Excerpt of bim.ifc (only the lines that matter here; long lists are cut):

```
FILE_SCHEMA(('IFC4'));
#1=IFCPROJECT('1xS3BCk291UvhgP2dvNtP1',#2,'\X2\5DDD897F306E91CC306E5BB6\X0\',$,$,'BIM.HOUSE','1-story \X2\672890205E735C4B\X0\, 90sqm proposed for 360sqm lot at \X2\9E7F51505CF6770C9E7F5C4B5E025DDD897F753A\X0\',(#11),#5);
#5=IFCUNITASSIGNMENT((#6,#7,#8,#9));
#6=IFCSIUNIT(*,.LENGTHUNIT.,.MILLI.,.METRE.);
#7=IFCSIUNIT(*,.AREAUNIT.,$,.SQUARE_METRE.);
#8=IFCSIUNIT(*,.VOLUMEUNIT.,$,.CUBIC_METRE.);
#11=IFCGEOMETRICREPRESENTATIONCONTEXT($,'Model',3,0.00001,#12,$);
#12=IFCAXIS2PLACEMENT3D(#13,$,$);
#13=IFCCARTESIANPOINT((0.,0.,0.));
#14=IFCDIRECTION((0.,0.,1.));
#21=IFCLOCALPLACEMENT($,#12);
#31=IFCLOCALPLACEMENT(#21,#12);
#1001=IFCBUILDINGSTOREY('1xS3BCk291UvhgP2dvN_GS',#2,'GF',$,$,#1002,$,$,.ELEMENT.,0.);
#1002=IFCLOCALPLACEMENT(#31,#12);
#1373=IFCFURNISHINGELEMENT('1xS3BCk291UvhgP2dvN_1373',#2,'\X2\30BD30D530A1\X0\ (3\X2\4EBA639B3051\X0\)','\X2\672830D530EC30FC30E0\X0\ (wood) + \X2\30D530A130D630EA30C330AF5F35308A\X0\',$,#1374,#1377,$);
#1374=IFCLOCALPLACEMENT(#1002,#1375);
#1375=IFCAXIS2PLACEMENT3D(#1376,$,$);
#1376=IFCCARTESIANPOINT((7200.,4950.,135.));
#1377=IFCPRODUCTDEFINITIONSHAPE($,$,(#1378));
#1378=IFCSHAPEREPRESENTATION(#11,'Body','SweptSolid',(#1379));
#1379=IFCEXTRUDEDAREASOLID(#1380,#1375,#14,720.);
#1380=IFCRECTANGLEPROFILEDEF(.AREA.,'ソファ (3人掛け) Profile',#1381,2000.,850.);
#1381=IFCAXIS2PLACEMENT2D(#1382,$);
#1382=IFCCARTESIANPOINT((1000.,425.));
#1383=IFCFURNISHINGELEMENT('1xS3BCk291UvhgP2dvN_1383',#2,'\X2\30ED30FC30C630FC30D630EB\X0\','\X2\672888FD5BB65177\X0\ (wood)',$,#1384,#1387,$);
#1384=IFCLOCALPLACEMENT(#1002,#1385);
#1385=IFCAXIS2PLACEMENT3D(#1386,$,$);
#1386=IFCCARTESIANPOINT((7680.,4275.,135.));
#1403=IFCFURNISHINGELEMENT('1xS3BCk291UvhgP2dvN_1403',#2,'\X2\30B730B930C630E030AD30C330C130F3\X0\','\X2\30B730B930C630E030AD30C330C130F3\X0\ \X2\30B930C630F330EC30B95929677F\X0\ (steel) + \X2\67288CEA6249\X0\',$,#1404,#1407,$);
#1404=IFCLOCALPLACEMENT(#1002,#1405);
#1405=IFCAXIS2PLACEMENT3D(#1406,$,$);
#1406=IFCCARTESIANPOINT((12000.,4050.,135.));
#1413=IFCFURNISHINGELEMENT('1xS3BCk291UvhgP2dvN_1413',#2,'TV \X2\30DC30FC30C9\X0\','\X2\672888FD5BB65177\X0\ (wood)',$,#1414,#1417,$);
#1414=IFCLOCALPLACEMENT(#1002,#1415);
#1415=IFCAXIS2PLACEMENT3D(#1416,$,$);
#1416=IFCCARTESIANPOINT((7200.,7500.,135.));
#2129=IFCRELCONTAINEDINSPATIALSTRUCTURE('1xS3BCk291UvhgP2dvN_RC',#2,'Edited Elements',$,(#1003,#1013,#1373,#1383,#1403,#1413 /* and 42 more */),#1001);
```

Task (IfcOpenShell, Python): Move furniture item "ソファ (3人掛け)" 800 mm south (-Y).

```python
import ifcopenshell
import ifcopenshell.api.geometry
import ifcopenshell.util.placement

model = ifcopenshell.open("bim.ifc")

item = model.by_guid("1xS3BCk291UvhgP2dvN_1373")
matrix = ifcopenshell.util.placement.get_local_placement(item.ObjectPlacement)
matrix[1, 3] -= 800.0
ifcopenshell.api.geometry.edit_object_placement(model, product=item, matrix=matrix, is_si=False)

print(ifcopenshell.util.placement.get_local_placement(item.ObjectPlacement).round(3) + 0.0)

model.write("bim_updated.ifc")
```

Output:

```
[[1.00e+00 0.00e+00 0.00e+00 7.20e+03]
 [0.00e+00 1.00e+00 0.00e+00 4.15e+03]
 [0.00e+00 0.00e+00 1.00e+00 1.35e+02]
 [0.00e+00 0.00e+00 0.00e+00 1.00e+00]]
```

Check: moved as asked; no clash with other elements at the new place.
